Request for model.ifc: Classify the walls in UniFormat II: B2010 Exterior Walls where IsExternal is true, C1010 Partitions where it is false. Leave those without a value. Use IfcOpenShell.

First a look at what the model holds.

```python
import ifcopenshell
import ifcopenshell.util.element

model = ifcopenshell.open("model.ifc")
print(model.schema)
print("classifications:", [c.Name for c in model.by_type("IfcClassification")])
values = [ifcopenshell.util.element.get_pset(e, "Pset_WallCommon", "IsExternal") for e in model.by_type("IfcWall")]
for value in (True, False, None):
    print("IsExternal", value, values.count(value))
```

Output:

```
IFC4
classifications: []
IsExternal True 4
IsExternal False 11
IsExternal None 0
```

```python
import ifcopenshell
import ifcopenshell.api.classification
import ifcopenshell.util.element

model = ifcopenshell.open("model.ifc")

system = ifcopenshell.api.classification.add_classification(model, classification="UniFormat II")

walls = model.by_type("IfcWall")
external = {e: ifcopenshell.util.element.get_pset(e, "Pset_WallCommon", "IsExternal") for e in walls}
for flag, code, name in ((True, "B2010", "Exterior Walls"), (False, "C1010", "Partitions")):
    products = [e for e in walls if external[e] is flag]
    ifcopenshell.api.classification.add_reference(
        model, products=products, classification=system, identification=code, name=name
    )
    print(code, len(products))

model.write("model_edited.ifc")
```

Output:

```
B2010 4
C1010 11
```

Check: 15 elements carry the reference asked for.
